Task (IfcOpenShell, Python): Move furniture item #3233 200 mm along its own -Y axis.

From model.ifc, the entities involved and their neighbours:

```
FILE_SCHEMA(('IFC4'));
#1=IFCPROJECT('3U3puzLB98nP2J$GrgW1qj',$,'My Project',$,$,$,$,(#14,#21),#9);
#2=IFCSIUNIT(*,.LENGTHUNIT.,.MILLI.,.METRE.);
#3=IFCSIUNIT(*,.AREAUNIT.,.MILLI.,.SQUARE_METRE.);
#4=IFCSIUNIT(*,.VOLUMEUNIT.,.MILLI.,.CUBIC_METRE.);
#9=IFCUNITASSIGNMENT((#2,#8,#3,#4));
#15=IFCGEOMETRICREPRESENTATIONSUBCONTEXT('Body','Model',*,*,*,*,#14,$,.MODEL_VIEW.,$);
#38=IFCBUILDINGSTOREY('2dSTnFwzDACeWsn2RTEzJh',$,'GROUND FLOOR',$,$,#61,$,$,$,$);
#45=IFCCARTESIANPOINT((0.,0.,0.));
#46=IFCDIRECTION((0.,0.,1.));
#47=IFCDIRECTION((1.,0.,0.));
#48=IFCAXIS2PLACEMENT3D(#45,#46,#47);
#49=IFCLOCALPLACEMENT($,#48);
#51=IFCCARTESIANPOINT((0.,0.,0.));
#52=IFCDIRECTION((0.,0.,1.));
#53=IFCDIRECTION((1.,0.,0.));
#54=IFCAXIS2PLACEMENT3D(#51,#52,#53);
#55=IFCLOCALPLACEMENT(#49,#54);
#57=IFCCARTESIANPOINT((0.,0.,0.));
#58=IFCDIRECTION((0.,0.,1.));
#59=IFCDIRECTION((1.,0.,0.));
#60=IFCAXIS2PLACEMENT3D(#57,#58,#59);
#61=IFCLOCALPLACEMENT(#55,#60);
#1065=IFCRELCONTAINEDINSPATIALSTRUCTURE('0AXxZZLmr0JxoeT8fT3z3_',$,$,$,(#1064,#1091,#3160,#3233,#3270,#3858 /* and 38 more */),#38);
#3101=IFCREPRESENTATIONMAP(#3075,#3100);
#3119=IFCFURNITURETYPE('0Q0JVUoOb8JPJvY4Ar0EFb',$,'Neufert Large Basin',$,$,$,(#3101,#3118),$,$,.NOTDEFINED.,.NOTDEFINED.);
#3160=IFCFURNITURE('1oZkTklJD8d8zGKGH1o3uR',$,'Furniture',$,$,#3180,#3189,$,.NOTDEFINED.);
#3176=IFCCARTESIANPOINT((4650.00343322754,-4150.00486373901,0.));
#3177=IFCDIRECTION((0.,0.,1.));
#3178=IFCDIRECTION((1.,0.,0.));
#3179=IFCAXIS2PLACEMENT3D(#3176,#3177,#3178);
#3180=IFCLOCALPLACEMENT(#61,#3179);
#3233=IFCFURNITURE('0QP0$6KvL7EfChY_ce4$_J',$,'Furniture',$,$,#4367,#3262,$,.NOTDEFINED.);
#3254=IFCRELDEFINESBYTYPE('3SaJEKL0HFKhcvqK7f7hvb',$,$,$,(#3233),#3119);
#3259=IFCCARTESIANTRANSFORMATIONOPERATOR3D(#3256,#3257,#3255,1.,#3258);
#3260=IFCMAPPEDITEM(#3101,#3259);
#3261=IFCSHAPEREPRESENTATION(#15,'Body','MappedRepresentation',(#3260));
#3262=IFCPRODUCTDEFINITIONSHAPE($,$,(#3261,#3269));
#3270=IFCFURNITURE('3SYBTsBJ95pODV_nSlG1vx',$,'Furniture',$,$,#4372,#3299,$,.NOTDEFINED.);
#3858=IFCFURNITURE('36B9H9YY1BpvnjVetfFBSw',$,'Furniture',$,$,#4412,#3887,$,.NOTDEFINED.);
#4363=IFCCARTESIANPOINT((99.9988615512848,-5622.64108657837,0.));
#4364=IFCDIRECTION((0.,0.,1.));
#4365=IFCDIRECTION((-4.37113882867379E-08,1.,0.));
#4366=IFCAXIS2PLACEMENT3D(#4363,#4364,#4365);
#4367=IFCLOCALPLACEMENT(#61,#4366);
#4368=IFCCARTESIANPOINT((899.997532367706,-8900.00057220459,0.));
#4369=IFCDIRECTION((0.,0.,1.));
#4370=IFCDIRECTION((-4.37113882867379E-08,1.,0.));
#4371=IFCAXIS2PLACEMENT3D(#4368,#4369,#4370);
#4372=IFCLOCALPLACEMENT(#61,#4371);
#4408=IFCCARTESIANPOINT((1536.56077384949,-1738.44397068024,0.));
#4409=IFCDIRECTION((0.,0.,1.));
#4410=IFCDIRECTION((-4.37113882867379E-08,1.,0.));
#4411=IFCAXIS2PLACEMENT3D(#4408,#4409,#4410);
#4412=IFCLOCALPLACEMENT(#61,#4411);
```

```python
import ifcopenshell
import ifcopenshell.api.geometry
import ifcopenshell.util.placement
import ifcopenshell.util.unit

model = ifcopenshell.open("model.ifc")
unit_scale = ifcopenshell.util.unit.calculate_unit_scale(model)

item = model.by_id(3233)
matrix = ifcopenshell.util.placement.get_local_placement(item.ObjectPlacement)
matrix[:3, 3] -= matrix[:3, 1] * 0.2 / unit_scale
ifcopenshell.api.geometry.edit_object_placement(model, product=item, matrix=matrix, is_si=False)

print(ifcopenshell.util.placement.get_local_placement(item.ObjectPlacement).round(3) + 0.0)

model.write("model_edited.ifc")
```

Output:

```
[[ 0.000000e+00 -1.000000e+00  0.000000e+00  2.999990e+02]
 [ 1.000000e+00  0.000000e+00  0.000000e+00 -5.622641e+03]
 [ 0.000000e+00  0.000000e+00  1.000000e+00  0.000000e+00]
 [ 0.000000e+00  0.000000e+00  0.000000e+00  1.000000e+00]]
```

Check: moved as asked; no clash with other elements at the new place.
